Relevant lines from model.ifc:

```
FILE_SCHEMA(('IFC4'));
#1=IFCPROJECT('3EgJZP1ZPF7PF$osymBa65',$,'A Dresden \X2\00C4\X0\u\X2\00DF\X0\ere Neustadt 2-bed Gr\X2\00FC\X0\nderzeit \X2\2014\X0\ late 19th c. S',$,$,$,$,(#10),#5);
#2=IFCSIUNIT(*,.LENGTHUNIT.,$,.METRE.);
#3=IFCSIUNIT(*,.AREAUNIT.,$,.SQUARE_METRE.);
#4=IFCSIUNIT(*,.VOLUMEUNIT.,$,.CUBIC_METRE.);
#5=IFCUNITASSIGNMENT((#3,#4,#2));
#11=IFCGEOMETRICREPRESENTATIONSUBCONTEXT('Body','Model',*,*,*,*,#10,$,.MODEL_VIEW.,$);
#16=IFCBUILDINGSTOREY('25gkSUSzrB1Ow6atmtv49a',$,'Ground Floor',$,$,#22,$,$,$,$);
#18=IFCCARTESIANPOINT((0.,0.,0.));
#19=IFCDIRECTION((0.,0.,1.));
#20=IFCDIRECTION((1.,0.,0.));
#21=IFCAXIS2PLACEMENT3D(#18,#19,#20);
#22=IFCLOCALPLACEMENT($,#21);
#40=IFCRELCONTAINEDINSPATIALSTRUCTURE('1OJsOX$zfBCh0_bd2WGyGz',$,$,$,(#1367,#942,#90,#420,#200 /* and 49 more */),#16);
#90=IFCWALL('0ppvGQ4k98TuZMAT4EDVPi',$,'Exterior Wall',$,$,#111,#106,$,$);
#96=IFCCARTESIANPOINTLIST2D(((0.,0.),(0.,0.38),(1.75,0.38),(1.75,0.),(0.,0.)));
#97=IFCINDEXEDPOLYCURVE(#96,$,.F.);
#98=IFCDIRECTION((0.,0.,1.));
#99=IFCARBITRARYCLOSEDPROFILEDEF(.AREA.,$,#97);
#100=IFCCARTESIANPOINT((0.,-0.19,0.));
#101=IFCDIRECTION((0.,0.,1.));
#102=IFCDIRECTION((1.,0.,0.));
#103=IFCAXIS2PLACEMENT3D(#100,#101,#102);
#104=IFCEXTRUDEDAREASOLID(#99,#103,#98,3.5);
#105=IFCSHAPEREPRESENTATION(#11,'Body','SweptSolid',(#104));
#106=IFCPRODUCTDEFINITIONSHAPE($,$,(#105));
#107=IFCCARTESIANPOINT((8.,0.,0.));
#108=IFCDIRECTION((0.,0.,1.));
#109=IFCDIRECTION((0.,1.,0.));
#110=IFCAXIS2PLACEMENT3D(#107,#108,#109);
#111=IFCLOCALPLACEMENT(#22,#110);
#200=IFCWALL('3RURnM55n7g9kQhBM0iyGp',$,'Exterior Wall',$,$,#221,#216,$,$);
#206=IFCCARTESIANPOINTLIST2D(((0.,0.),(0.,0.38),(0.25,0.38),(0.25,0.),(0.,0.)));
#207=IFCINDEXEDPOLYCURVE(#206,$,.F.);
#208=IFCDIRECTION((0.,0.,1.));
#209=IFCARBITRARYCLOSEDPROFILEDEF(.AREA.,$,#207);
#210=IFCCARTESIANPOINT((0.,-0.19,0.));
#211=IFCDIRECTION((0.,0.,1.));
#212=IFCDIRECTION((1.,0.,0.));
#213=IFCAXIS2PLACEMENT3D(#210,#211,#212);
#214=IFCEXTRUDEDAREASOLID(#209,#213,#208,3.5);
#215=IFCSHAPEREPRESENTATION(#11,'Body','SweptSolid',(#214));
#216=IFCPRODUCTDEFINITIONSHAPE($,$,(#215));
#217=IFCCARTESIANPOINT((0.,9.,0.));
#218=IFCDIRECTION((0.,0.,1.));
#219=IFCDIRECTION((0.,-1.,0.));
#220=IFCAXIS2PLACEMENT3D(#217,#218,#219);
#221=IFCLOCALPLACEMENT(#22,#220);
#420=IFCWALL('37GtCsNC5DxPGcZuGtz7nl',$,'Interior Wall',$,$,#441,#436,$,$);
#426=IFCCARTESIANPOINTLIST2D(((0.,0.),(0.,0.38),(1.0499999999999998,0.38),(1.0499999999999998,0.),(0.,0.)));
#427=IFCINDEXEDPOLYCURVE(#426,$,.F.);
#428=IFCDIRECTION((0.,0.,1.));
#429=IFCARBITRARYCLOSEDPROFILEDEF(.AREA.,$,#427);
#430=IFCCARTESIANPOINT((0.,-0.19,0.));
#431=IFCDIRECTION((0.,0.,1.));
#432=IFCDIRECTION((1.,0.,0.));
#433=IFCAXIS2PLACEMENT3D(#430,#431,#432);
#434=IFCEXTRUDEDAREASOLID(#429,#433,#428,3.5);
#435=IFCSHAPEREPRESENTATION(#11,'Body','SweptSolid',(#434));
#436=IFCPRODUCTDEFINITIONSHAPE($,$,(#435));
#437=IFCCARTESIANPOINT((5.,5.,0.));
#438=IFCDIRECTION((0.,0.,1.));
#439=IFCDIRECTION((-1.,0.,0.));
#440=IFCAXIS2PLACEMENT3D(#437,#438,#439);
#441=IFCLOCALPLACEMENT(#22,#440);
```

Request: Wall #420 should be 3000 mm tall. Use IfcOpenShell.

```python
import ifcopenshell
import ifcopenshell.geom
import ifcopenshell.util.representation
import ifcopenshell.util.shape
import ifcopenshell.util.unit

model = ifcopenshell.open("model.ifc")
unit_scale = ifcopenshell.util.unit.calculate_unit_scale(model)
settings = ifcopenshell.geom.settings()


def volume(element):
    """Net volume in cubic metres, openings subtracted."""
    shape = ifcopenshell.geom.create_shape(settings, element)
    return ifcopenshell.util.shape.get_volume(shape.geometry)


wall = model.by_id(420)
before = volume(wall)

body = ifcopenshell.util.representation.get_representation(wall, "Model", "Body")
solid = body.Items[0]
old_height = solid.Depth
solid.Depth = 3 / unit_scale
after = volume(wall)

print(f"height {old_height:g} -> {solid.Depth:g}, volume {before:.3f} -> {after:.3f} m3")

model.write("model_v2.ifc")
```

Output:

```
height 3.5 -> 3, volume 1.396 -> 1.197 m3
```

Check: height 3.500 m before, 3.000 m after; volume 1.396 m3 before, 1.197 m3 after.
